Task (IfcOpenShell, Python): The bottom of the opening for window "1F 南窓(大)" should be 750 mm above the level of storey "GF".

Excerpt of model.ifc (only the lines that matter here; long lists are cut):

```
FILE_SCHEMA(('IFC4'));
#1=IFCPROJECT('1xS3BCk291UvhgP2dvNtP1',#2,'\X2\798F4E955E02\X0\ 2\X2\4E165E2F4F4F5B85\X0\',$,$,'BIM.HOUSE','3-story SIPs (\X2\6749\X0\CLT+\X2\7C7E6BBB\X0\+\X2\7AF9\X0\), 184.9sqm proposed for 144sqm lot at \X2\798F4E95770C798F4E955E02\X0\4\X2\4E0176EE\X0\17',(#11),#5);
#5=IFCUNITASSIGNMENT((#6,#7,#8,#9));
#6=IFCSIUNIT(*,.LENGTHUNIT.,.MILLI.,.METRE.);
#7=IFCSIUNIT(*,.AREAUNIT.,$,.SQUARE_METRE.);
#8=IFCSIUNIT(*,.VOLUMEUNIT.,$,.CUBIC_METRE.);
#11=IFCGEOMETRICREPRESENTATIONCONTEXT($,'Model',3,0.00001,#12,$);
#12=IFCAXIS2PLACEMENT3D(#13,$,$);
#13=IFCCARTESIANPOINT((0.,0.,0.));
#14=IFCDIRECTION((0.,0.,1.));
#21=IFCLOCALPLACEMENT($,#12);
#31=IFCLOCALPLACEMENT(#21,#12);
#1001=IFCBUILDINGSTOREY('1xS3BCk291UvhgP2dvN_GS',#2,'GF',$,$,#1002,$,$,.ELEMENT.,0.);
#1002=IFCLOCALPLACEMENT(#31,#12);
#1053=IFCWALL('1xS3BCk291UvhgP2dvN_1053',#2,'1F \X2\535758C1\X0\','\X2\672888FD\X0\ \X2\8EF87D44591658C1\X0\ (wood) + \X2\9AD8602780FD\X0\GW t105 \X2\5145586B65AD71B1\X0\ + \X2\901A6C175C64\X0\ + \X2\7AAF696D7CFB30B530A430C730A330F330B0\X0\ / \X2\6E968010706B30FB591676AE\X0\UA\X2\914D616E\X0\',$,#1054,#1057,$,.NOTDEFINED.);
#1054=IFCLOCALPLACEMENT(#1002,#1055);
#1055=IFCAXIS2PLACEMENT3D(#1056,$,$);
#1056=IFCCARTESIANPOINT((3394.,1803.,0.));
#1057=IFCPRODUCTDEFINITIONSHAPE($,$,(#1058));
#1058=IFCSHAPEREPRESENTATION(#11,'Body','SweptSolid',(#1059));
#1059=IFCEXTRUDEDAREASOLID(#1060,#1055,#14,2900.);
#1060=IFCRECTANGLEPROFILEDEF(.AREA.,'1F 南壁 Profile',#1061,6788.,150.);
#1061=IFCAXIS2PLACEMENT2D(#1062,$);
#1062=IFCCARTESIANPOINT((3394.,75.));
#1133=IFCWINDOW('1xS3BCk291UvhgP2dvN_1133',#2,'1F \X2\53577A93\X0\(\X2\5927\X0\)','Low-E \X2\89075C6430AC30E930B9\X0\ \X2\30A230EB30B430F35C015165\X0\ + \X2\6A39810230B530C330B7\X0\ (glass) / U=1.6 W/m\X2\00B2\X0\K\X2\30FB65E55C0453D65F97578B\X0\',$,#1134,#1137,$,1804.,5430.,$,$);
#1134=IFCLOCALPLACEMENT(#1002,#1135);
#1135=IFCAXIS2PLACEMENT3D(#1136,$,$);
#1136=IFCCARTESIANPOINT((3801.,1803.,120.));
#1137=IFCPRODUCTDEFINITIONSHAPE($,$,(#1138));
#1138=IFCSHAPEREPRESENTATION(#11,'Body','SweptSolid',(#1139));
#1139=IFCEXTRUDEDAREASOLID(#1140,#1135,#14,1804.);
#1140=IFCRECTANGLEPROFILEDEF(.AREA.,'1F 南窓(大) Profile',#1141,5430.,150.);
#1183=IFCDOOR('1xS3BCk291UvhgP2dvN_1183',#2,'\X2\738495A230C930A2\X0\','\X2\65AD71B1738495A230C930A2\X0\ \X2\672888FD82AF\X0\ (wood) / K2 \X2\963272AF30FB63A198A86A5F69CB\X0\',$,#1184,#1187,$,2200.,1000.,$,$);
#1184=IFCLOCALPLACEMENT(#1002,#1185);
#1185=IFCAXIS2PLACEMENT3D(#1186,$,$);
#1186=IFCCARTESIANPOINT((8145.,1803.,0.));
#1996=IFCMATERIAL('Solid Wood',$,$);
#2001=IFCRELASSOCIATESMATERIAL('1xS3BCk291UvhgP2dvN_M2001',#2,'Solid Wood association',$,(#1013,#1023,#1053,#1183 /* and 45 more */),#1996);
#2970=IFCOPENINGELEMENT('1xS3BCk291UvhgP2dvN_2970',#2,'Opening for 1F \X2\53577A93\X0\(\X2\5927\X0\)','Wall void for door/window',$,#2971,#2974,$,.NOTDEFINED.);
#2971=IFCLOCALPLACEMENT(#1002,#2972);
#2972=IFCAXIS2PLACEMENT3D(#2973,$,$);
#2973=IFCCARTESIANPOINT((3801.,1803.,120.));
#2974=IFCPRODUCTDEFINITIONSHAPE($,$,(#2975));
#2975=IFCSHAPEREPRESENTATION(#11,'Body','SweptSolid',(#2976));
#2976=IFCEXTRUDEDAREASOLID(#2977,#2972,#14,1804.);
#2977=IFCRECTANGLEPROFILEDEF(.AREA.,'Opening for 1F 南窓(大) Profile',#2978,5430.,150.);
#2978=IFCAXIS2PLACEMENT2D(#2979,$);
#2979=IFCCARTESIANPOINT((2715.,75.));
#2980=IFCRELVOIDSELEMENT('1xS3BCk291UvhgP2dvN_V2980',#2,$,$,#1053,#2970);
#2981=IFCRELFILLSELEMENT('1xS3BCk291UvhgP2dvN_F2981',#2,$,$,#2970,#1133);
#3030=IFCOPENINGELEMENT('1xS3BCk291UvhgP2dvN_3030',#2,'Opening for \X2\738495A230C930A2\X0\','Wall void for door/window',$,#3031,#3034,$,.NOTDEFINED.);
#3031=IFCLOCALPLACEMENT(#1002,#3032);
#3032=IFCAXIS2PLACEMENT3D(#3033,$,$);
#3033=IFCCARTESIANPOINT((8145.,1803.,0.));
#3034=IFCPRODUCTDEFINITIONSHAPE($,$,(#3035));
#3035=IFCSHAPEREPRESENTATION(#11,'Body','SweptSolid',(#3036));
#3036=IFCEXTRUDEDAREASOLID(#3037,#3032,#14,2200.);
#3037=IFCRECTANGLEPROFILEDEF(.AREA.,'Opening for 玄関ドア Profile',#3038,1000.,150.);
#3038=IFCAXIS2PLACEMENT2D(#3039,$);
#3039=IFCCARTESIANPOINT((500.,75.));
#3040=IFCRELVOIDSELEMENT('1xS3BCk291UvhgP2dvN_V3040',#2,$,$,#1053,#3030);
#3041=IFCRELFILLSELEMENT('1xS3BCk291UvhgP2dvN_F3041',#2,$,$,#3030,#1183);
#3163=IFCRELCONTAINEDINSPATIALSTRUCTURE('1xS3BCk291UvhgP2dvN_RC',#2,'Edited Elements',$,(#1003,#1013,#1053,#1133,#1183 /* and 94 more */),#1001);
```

```python
import numpy as np
import ifcopenshell
import ifcopenshell.api.geometry
import ifcopenshell.geom
import ifcopenshell.util.element
import ifcopenshell.util.placement
import ifcopenshell.util.shape
import ifcopenshell.util.unit

model = ifcopenshell.open("model.ifc")
unit_scale = ifcopenshell.util.unit.calculate_unit_scale(model)

window = model.by_guid("1xS3BCk291UvhgP2dvN_1133")
opening = window.FillsVoids[0].RelatingOpeningElement
storey = ifcopenshell.util.element.get_container(window, ifc_class="IfcBuildingStorey")
level = ifcopenshell.util.placement.get_local_placement(storey.ObjectPlacement)[2, 3]

# The opening's origin need not be at the sill, so measure its lowest point.
shape = ifcopenshell.geom.create_shape(ifcopenshell.geom.settings(), opening)
bottom = ifcopenshell.util.shape.get_shape_bottom_elevation(shape, shape.geometry) / unit_scale
dz = level + 750.0 - bottom

shift = np.array([0.0, 0.0, dz])
# The window is not placed relative to its opening, so move both.
for product in (opening, window):
    matrix = ifcopenshell.util.placement.get_local_placement(product.ObjectPlacement)
    matrix[:3, 3] += shift
    ifcopenshell.api.geometry.edit_object_placement(model, product=product, matrix=matrix, is_si=False)

print(f"moved by {dz * unit_scale:+.3f} m")

model.write("model-out.ifc")
```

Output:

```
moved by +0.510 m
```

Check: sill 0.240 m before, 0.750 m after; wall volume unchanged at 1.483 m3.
